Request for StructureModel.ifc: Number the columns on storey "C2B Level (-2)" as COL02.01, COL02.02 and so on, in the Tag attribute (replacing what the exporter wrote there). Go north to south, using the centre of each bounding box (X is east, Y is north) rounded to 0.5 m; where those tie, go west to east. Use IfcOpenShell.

First a look at what the model holds.

```python
import ifcopenshell
import ifcopenshell.util.element
import ifcopenshell.util.placement

model = ifcopenshell.open("StructureModel.ifc")
print(model.schema)
storey = next(s for s in model.by_type("IfcBuildingStorey") if s.Name == "C2B Level (-2)")
columns = [e for e in ifcopenshell.util.element.get_decomposition(storey) if e.is_a("IfcColumn")]
for e in sorted(columns, key=lambda e: e.id()):
    origin = ifcopenshell.util.placement.get_local_placement(e.ObjectPlacement)[:3, 3]
    print(e.id(), e.Tag, e.Name, origin.round(2) + 0.0, sep=" | ")
```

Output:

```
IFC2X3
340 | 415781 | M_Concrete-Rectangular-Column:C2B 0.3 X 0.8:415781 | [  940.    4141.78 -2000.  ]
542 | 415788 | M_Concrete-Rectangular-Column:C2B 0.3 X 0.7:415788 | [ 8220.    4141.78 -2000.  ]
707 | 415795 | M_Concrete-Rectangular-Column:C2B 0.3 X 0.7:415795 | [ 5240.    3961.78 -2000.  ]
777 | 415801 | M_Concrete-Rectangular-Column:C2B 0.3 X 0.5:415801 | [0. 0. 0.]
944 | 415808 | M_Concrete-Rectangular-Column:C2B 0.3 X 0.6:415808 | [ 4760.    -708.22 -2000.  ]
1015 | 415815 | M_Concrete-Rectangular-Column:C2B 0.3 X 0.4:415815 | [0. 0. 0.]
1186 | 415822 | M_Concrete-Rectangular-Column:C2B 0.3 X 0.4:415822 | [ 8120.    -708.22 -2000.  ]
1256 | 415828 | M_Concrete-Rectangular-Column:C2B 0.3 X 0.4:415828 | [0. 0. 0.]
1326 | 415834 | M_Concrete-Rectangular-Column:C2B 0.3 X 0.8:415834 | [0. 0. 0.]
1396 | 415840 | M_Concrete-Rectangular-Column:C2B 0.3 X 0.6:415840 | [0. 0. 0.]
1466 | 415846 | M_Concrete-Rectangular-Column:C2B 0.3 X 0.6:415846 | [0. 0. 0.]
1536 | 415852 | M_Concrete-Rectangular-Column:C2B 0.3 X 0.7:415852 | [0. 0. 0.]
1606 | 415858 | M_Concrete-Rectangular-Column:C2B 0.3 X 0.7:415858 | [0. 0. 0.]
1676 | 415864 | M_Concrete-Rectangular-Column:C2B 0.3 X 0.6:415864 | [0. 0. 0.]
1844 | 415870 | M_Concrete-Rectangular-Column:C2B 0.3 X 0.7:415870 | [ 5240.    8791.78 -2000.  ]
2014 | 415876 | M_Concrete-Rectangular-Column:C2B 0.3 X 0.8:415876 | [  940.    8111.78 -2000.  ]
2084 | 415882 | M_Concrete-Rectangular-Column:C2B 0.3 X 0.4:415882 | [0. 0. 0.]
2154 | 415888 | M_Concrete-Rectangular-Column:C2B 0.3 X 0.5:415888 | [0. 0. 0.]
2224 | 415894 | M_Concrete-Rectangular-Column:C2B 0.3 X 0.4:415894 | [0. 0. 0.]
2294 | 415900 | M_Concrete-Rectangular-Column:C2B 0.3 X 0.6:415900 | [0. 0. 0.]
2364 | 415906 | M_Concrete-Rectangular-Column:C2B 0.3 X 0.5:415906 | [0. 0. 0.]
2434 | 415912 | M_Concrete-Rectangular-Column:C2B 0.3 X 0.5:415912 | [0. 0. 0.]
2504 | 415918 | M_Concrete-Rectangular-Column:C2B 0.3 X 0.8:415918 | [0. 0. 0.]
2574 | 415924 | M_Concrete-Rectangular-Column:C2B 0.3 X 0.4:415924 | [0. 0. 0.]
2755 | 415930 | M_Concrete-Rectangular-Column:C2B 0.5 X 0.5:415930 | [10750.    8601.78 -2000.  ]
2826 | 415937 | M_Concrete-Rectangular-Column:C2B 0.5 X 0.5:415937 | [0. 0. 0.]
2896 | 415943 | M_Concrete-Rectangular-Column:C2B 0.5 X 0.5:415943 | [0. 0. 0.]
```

```python
import ifcopenshell
import ifcopenshell.geom
import ifcopenshell.util.element
import ifcopenshell.util.shape

model = ifcopenshell.open("StructureModel.ifc")
settings = ifcopenshell.geom.settings()
settings.set("use-world-coords", True)


def centre(element):
    shape = ifcopenshell.geom.create_shape(settings, element)
    return ifcopenshell.util.shape.get_bbox_centroid(shape.geometry)


storey = next(s for s in model.by_type("IfcBuildingStorey") if s.Name == "C2B Level (-2)")
columns = [e for e in ifcopenshell.util.element.get_decomposition(storey) if e.is_a("IfcColumn")]

# Insertion points can sit at a corner or the storey origin, so sort by the geometry (in metres).
centres = {e: centre(e) for e in columns}
columns.sort(key=lambda e: (-round(centres[e][1] / 0.5), centres[e][0]))

for i, e in enumerate(columns, start=1):
    number = f"COL02.{i:02d}"
    e.Tag = number
    print(e.id(), number)

model.write("StructureModel_updated.ifc")
```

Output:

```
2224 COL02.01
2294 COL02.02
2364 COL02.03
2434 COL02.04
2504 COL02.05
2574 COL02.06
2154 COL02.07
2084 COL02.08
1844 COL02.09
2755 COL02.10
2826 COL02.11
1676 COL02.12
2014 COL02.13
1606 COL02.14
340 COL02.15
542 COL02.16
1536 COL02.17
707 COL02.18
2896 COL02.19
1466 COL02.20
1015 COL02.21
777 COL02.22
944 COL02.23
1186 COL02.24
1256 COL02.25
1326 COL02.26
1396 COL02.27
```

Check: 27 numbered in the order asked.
